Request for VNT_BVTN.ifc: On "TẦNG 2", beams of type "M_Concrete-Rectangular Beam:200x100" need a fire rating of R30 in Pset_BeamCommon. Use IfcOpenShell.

First a look at what the model holds.

```python
import ifcopenshell
import ifcopenshell.util.element

model = ifcopenshell.open("VNT_BVTN.ifc")
print(model.schema)
storey = next(s for s in model.by_type("IfcBuildingStorey") if s.Name == "TẦNG 2")
beams = [e for e in ifcopenshell.util.element.get_decomposition(storey) if e.is_a("IfcBeam")]
seen = {}
for e in beams:
    element_type = ifcopenshell.util.element.get_type(e)
    key = (element_type.Name if element_type != e and element_type else None, ifcopenshell.util.element.get_pset(e, "Pset_BeamCommon", "FireRating"))
    seen[key] = seen.get(key, 0) + 1
for (name, value), count in sorted(seen.items(), key=str):
    print(count, "x", name, "|", value)
```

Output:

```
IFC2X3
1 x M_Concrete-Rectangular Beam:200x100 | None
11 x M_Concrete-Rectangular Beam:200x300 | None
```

```python
import ifcopenshell
import ifcopenshell.api.pset
import ifcopenshell.util.element

model = ifcopenshell.open("VNT_BVTN.ifc")

storey = next(s for s in model.by_type("IfcBuildingStorey") if s.Name == "TẦNG 2")
beams = [e for e in ifcopenshell.util.element.get_decomposition(storey) if e.is_a("IfcBeam")]

count = 0
for e in beams:
    element_type = ifcopenshell.util.element.get_type(e)
    if element_type in (None, e) or element_type.Name != "M_Concrete-Rectangular Beam:200x100":
        continue
    # add_pset returns the element's existing set when there is one.
    pset = ifcopenshell.api.pset.add_pset(model, product=e, name="Pset_BeamCommon")
    ifcopenshell.api.pset.edit_pset(model, pset=pset, properties={"FireRating": "R30"})
    count += 1

print(count, "beams updated")

model.write("VNT_BVTN_rev.ifc")
```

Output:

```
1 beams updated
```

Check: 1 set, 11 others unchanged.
